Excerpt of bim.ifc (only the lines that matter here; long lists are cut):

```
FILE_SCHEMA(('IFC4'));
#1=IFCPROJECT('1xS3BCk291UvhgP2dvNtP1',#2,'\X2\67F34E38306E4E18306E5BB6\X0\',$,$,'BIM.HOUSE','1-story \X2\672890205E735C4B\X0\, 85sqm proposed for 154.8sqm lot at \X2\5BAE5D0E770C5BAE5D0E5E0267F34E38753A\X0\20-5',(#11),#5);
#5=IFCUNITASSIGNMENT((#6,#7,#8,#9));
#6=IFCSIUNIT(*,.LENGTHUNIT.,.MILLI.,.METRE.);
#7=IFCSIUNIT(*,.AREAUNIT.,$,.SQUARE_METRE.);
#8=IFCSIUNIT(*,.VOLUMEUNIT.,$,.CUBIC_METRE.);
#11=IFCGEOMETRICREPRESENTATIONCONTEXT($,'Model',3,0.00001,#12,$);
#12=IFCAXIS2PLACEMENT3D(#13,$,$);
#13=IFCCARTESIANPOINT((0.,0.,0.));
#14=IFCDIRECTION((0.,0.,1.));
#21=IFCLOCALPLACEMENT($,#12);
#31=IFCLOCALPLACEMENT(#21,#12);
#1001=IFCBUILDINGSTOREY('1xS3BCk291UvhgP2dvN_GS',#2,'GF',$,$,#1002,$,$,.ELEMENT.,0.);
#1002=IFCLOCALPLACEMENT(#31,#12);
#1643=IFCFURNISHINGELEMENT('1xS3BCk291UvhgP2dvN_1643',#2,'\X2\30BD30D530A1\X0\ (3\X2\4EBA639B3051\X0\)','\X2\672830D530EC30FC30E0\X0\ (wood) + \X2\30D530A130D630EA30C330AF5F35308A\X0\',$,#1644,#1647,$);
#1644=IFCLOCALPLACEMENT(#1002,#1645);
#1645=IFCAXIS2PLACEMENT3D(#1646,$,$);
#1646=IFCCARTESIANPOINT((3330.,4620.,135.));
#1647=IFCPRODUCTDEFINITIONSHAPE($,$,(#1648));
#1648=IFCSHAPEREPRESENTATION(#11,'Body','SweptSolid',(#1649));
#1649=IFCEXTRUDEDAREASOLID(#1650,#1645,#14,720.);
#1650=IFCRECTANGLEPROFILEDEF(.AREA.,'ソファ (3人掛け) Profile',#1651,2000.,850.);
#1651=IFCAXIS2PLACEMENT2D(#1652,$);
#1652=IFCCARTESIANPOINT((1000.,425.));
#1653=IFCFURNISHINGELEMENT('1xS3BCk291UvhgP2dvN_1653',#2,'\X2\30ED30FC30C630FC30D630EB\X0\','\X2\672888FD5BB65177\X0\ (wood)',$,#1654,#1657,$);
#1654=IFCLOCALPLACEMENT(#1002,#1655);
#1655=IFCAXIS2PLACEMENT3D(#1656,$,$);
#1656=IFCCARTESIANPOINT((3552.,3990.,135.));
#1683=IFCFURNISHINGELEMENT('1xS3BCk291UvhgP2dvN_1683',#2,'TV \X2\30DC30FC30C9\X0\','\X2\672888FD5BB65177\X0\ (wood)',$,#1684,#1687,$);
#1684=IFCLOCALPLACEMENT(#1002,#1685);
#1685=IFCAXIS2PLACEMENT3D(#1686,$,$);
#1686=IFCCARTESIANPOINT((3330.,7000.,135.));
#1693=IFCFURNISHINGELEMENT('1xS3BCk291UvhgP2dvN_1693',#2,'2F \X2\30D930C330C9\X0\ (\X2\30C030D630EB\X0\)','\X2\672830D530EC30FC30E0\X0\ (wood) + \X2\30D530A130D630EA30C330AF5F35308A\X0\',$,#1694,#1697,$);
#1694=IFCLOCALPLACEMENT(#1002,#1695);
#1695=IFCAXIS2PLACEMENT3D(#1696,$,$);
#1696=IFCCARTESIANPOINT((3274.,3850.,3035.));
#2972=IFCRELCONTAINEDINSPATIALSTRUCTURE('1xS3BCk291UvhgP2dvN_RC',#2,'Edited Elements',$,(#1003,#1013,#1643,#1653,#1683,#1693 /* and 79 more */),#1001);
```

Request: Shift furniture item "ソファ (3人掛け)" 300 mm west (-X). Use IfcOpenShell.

```python
import ifcopenshell
import ifcopenshell.api.geometry
import ifcopenshell.util.placement
import ifcopenshell.util.unit

model = ifcopenshell.open("bim.ifc")
unit_scale = ifcopenshell.util.unit.calculate_unit_scale(model)

item = model.by_guid("1xS3BCk291UvhgP2dvN_1643")
matrix = ifcopenshell.util.placement.get_local_placement(item.ObjectPlacement)
matrix[0, 3] -= 0.3 / unit_scale
ifcopenshell.api.geometry.edit_object_placement(model, product=item, matrix=matrix, is_si=False)

print(ifcopenshell.util.placement.get_local_placement(item.ObjectPlacement).round(3) + 0.0)

model.write("bim_edited.ifc")
```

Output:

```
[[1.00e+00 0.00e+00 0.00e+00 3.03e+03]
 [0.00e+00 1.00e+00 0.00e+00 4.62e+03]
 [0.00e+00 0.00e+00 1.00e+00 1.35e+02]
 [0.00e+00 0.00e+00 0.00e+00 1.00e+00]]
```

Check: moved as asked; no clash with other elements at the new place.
